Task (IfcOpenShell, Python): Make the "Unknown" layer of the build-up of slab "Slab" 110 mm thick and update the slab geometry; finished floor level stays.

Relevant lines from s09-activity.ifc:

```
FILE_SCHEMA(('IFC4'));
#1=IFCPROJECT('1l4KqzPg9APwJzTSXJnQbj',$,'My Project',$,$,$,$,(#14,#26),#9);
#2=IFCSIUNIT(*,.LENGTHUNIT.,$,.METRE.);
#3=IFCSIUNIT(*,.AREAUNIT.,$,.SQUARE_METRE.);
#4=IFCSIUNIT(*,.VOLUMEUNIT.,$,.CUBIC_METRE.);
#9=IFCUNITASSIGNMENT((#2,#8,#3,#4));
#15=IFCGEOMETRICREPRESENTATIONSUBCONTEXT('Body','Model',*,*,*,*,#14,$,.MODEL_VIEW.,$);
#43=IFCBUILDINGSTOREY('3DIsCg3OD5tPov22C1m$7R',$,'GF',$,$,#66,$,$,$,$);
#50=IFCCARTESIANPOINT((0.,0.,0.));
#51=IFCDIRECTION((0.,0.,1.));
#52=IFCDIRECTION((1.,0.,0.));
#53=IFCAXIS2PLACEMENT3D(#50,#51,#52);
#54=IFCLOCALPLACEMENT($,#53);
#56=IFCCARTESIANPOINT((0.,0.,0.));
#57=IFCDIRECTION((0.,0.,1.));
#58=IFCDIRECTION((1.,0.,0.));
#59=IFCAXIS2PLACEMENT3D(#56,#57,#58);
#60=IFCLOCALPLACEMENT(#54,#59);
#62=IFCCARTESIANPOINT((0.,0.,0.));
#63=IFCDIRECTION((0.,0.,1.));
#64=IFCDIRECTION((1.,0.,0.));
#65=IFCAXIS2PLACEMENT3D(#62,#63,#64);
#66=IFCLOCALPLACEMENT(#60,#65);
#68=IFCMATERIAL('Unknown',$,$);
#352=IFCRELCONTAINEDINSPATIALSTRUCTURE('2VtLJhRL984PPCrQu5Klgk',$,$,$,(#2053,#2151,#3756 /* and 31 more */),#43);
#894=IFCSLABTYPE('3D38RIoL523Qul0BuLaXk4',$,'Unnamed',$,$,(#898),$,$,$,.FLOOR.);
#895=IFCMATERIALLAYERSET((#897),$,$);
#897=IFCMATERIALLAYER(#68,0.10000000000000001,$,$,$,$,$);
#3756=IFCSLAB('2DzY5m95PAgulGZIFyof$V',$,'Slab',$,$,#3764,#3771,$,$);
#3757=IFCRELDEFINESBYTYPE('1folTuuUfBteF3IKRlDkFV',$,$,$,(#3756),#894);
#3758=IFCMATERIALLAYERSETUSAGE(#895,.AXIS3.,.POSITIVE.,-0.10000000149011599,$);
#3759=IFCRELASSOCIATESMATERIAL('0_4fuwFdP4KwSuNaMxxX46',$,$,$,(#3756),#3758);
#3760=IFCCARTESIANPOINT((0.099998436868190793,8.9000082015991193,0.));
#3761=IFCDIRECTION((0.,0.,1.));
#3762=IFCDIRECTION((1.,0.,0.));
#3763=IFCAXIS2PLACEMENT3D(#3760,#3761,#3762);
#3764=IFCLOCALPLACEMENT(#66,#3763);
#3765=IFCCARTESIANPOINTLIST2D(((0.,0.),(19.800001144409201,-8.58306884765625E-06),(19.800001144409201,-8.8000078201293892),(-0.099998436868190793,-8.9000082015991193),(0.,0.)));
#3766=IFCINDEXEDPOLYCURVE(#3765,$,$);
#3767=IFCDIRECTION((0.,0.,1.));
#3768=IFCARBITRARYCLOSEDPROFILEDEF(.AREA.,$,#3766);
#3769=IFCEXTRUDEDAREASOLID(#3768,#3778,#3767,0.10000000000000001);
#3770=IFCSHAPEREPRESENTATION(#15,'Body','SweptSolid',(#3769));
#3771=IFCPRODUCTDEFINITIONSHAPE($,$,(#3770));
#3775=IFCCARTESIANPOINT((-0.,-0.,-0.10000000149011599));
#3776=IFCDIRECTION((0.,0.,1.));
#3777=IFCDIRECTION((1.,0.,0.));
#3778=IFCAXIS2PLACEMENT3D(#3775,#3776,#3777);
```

```python
import ifcopenshell
import ifcopenshell.util.element
import ifcopenshell.util.representation
import ifcopenshell.util.unit

model = ifcopenshell.open("s09-activity.ifc")
unit_scale = ifcopenshell.util.unit.calculate_unit_scale(model)

layer_set = model.by_id(895)
layer = next(l for l in layer_set.MaterialLayers if l.Material and l.Material.Name == "Unknown")
change = 0.11 / unit_scale - layer.LayerThickness
layer.LayerThickness += change

# Geometry does not follow the layer set by itself.
slabs = [e for e in ifcopenshell.util.element.get_elements_by_material(model, layer_set) if e.is_a("IfcSlab")]
for slab in sorted(slabs, key=lambda e: e.id()):
    body = ifcopenshell.util.representation.get_representation(slab, "Model", "Body")
    solid = body.Items[0]
    old_depth = solid.Depth
    solid.Depth += change
    # Extruded upwards: lower the start of the extrusion so the top stays.
    x, y, z = solid.Position.Location.Coordinates
    solid.Position.Location = model.createIfcCartesianPoint((x, y, z - change))
    print(slab.id(), f"{old_depth:g} -> {solid.Depth:g}")

# The layers are counted up from the underside, which has moved.
for usage in {ifcopenshell.util.element.get_material(slab) for slab in slabs}:
    usage.OffsetFromReferenceLine -= change

model.write("s09-activity-out.ifc")
```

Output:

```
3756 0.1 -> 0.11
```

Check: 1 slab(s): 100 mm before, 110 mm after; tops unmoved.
